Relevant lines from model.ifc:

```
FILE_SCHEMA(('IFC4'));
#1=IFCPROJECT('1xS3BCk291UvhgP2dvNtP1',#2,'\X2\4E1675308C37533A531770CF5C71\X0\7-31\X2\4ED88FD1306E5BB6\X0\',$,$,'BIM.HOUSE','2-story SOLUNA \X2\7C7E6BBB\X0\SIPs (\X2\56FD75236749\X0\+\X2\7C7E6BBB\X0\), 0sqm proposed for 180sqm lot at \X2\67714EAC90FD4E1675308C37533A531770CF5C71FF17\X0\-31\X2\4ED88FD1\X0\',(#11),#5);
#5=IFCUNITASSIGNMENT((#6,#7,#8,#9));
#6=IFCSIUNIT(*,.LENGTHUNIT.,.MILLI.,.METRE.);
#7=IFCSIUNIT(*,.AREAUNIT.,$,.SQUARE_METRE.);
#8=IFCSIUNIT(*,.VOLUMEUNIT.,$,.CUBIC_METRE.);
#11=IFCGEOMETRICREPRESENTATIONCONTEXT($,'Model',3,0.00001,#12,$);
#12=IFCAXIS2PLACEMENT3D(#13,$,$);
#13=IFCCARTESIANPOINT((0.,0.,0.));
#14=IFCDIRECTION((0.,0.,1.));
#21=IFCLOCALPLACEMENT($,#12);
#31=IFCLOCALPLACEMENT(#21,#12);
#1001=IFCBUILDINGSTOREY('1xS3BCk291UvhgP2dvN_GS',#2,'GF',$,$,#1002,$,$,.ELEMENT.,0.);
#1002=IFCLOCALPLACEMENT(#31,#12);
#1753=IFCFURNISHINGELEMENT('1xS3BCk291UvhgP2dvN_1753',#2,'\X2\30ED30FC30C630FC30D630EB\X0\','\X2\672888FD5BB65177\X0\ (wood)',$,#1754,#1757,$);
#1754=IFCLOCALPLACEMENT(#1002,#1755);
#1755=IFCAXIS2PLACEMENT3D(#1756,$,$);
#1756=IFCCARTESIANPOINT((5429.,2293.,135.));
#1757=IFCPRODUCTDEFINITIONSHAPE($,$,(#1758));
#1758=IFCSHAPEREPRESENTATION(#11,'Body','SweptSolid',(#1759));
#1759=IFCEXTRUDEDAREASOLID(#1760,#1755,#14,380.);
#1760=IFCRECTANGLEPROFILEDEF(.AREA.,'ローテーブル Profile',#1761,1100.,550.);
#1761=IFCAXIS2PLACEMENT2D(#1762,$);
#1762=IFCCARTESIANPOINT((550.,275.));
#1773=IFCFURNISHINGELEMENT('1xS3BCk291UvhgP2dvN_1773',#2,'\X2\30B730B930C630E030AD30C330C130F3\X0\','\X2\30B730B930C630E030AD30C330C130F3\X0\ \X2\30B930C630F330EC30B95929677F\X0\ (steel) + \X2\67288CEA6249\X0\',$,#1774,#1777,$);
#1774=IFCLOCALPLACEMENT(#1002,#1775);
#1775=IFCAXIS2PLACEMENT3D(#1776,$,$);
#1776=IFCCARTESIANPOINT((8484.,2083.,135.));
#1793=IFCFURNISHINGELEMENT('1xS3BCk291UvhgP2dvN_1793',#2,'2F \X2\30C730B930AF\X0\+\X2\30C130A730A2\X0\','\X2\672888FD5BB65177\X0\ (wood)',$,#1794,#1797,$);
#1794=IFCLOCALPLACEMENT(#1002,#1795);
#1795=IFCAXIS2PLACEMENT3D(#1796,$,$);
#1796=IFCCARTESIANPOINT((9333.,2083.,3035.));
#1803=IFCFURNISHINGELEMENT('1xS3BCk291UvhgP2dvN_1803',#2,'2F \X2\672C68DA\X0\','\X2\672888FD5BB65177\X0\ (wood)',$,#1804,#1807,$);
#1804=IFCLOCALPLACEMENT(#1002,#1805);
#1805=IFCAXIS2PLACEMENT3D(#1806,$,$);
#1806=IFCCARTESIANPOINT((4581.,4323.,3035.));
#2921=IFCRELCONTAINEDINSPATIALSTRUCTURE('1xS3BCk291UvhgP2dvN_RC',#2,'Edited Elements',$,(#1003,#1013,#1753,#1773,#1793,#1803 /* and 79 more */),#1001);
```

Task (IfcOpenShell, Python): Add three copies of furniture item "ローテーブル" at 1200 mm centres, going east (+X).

```python
import numpy as np
import ifcopenshell
import ifcopenshell.api.geometry
import ifcopenshell.api.root
import ifcopenshell.util.element
import ifcopenshell.util.placement

model = ifcopenshell.open("model.ifc")


def reuse_history(source, copy):
    """copy_class also copies each property set's owner history, people and application; keep the originals."""
    for rel in copy.IsDefinedBy:
        if rel.is_a("IfcRelDefinesByProperties") and (history := rel.RelatingPropertyDefinition.OwnerHistory):
            rel.RelatingPropertyDefinition.OwnerHistory = source.OwnerHistory
            ifcopenshell.util.element.remove_deep2(model, history)


source = model.by_id(1753)
base = ifcopenshell.util.placement.get_local_placement(source.ObjectPlacement)
step = np.array([1.0, 0.0, 0.0]) * 1200.0

for i in range(1, 4):
    copy = ifcopenshell.api.root.copy_class(model, product=source)
    copy.Representation = ifcopenshell.util.element.copy_deep(
        model, source.Representation, exclude=["IfcGeometricRepresentationContext", "IfcRepresentationMap"]
    )
    reuse_history(source, copy)
    matrix = base.copy()
    matrix[:3, 3] += i * step
    print("added at", matrix[:3, 3].round(3) + 0.0)
    ifcopenshell.api.geometry.edit_object_placement(model, product=copy, matrix=matrix, is_si=False)

model.write("model_v2.ifc")
```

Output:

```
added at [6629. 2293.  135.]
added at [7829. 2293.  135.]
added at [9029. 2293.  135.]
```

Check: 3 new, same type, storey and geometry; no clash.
